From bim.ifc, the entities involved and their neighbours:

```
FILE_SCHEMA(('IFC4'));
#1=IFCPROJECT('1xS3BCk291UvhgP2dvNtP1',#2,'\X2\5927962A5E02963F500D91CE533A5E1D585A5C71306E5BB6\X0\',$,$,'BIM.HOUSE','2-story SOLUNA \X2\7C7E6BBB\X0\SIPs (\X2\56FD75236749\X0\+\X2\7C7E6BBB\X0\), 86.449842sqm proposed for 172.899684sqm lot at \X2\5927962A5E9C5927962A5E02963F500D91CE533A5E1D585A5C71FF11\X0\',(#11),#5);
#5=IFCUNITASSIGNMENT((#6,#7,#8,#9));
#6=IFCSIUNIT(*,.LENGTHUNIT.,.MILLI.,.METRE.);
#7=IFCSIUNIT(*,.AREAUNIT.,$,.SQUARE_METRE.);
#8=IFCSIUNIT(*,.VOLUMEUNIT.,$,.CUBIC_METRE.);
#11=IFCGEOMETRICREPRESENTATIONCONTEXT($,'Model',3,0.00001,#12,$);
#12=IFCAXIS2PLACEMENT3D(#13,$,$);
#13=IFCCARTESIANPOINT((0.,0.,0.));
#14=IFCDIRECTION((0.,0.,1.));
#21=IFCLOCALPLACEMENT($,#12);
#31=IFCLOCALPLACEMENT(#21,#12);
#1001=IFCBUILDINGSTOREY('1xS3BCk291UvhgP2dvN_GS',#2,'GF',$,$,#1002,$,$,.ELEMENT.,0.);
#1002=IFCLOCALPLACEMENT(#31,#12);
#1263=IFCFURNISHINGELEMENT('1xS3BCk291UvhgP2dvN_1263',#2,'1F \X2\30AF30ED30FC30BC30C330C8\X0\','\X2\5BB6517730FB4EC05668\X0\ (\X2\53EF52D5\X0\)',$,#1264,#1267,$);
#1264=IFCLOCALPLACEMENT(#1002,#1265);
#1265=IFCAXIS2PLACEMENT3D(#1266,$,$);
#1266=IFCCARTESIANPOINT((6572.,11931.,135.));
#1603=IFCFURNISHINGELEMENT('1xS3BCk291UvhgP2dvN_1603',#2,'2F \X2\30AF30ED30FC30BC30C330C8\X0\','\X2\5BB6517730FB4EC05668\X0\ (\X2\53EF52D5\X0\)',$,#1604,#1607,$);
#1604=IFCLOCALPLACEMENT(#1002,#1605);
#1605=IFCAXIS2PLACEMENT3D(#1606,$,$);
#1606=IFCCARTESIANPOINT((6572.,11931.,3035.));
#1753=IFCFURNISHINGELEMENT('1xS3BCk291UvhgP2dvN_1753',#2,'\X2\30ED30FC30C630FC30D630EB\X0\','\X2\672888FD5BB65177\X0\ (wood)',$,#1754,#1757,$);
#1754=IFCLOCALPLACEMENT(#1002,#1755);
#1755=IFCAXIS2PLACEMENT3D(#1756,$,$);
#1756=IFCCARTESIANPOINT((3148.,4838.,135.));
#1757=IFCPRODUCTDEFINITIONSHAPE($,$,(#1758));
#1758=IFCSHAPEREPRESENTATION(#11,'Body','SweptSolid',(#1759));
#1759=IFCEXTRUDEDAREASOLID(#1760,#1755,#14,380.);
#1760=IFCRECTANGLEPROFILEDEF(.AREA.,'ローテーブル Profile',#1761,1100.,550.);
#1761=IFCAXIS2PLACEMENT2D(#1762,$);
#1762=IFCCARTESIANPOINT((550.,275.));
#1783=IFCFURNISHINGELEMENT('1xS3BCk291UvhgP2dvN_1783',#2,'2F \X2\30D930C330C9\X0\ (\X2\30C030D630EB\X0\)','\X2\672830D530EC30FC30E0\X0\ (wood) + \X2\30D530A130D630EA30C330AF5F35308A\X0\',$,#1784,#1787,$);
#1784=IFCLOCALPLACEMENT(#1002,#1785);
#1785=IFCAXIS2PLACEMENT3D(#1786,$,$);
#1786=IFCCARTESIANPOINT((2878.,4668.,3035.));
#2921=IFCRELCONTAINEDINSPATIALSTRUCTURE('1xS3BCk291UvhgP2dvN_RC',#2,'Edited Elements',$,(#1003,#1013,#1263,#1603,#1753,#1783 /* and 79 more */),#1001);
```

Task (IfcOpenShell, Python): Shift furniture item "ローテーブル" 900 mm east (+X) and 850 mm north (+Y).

```python
import ifcopenshell
import ifcopenshell.api.geometry
import ifcopenshell.util.placement
import ifcopenshell.util.unit

model = ifcopenshell.open("bim.ifc")
unit_scale = ifcopenshell.util.unit.calculate_unit_scale(model)

item = model.by_id(1753)
matrix = ifcopenshell.util.placement.get_local_placement(item.ObjectPlacement)
matrix[0, 3] += 0.9 / unit_scale
matrix[1, 3] += 0.85 / unit_scale
ifcopenshell.api.geometry.edit_object_placement(model, product=item, matrix=matrix, is_si=False)

print(ifcopenshell.util.placement.get_local_placement(item.ObjectPlacement).round(3) + 0.0)

model.write("bim-out.ifc")
```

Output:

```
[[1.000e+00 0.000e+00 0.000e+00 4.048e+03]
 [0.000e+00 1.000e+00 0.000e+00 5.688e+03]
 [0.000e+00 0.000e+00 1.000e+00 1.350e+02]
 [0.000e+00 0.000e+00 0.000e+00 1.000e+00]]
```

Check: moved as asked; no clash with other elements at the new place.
